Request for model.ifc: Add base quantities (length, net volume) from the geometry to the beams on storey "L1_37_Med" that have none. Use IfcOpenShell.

First a look at what the model holds.

```python
import ifcopenshell
import ifcopenshell.util.element
import ifcopenshell.util.unit

model = ifcopenshell.open("model.ifc")
print(model.schema)
for unit_type in ("LENGTHUNIT", "AREAUNIT", "VOLUMEUNIT"):
    print(unit_type, ifcopenshell.util.unit.calculate_unit_scale(model, unit_type))
storey = next(s for s in model.by_type("IfcBuildingStorey") if s.Name == "L1_37_Med")
beams = [e for e in ifcopenshell.util.element.get_decomposition(storey) if e.is_a("IfcBeam")]
for e in sorted(beams, key=lambda e: e.id()):
    print(e.id(), e.is_a(), e.Name, list(ifcopenshell.util.element.get_psets(e, qtos_only=True)), sep=" | ")
```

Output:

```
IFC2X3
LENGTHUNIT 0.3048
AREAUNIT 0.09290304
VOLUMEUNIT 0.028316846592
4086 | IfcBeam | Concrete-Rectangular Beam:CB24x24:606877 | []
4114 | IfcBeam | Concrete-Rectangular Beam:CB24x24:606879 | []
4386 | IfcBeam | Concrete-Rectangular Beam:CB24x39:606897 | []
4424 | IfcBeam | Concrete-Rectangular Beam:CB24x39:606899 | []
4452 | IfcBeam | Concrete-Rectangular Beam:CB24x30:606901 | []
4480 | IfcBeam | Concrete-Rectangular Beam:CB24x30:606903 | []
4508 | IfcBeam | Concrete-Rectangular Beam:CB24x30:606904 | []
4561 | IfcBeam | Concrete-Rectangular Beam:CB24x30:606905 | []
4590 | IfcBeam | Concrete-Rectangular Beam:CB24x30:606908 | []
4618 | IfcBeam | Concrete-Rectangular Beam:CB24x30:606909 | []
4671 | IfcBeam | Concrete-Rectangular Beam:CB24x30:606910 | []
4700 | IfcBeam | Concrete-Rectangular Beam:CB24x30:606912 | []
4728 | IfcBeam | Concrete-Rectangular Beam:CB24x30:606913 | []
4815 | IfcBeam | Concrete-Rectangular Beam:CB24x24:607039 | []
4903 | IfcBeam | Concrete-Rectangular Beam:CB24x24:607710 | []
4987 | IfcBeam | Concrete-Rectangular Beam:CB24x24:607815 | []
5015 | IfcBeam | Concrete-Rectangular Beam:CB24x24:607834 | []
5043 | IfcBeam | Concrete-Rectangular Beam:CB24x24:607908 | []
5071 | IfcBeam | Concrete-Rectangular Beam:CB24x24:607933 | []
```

```python
import ifcopenshell
import ifcopenshell.api.pset
import ifcopenshell.geom
import ifcopenshell.util.element
import ifcopenshell.util.shape
import ifcopenshell.util.unit

model = ifcopenshell.open("model.ifc")
unit_scale = ifcopenshell.util.unit.calculate_unit_scale(model)
volume_scale = ifcopenshell.util.unit.calculate_unit_scale(model, "VOLUMEUNIT")
settings = ifcopenshell.geom.settings()

storey = next(s for s in model.by_type("IfcBuildingStorey") if s.Name == "L1_37_Med")
beams = [e for e in ifcopenshell.util.element.get_decomposition(storey) if e.is_a("IfcBeam")]

for e in sorted(beams, key=lambda e: e.id()):
    if ifcopenshell.util.element.get_psets(e, qtos_only=True, should_inherit=False):
        continue
    # Geometry comes back in metres, in the element's own axes.
    shape = ifcopenshell.geom.create_shape(settings, e)
    values = {
        "Length": ifcopenshell.util.shape.get_max_xyz(shape.geometry) / unit_scale,
        "NetVolume": ifcopenshell.util.shape.get_volume(shape.geometry) / volume_scale,
    }
    qto = ifcopenshell.api.pset.add_qto(model, product=e, name="BaseQuantities")
    ifcopenshell.api.pset.edit_qto(model, qto=qto, properties=values)
    print(e.id(), {k: round(v, 3) for k, v in values.items()})

model.write("model_updated.ifc")
```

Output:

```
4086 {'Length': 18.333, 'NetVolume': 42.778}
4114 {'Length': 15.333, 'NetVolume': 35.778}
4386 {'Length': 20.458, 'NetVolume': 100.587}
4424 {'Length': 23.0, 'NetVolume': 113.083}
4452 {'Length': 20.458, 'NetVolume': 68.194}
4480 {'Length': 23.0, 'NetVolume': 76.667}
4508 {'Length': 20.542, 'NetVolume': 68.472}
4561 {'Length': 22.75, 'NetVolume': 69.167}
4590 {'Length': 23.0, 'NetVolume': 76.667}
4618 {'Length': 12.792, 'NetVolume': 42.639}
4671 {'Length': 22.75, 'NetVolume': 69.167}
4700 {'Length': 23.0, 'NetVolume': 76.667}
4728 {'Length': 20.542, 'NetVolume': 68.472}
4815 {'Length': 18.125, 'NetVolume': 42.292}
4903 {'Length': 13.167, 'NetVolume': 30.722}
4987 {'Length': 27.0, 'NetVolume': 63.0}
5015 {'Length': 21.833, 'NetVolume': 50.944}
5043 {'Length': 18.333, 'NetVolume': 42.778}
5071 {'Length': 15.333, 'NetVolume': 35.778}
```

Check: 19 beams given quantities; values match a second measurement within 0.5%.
